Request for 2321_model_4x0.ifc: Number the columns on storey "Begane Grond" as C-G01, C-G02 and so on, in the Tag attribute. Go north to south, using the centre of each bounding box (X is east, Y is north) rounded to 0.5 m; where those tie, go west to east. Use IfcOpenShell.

First a look at what the model holds.

```python
import ifcopenshell
import ifcopenshell.util.element
import ifcopenshell.util.placement

model = ifcopenshell.open("2321_model_4x0.ifc")
print(model.schema)
storey = next(s for s in model.by_type("IfcBuildingStorey") if s.Name == "Begane Grond")
columns = [e for e in ifcopenshell.util.element.get_decomposition(storey) if e.is_a("IfcColumn")]
for e in sorted(columns, key=lambda e: e.id()):
    origin = ifcopenshell.util.placement.get_local_placement(e.ObjectPlacement)[:3, 3]
    print(e.id(), e.Tag, e.Name, origin.round(2) + 0.0, sep=" | ")
```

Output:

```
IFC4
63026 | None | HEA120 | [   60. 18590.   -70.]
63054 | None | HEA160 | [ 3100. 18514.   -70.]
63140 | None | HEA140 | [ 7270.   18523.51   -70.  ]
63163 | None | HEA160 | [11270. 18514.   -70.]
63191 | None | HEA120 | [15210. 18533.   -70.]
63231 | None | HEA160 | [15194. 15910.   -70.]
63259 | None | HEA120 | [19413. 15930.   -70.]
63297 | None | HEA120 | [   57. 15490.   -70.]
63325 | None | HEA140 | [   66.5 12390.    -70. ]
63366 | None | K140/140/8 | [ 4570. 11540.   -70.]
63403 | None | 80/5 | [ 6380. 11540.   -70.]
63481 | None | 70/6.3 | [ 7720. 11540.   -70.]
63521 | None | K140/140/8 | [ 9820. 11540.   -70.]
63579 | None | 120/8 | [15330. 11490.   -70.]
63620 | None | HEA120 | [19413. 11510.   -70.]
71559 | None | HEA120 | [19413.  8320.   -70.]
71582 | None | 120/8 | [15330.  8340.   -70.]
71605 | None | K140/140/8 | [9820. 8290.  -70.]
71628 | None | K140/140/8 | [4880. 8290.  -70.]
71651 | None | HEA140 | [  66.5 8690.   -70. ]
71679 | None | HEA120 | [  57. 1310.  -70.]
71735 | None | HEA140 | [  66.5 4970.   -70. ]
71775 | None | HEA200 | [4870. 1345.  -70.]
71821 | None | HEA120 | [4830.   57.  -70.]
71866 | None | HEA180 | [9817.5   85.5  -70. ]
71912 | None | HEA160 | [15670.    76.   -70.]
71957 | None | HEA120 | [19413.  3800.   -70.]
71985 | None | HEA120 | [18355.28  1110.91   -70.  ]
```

```python
import ifcopenshell
import ifcopenshell.geom
import ifcopenshell.util.element
import ifcopenshell.util.shape

model = ifcopenshell.open("2321_model_4x0.ifc")
settings = ifcopenshell.geom.settings()
settings.set("use-world-coords", True)


def centre(element):
    shape = ifcopenshell.geom.create_shape(settings, element)
    return ifcopenshell.util.shape.get_bbox_centroid(shape.geometry)


storey = next(s for s in model.by_type("IfcBuildingStorey") if s.Name == "Begane Grond")
columns = [e for e in ifcopenshell.util.element.get_decomposition(storey) if e.is_a("IfcColumn")]

# Insertion points can sit at a corner or the storey origin, so sort by the geometry (in metres).
centres = {e: centre(e) for e in columns}
columns.sort(key=lambda e: (-round(centres[e][1] / 0.5), centres[e][0]))

for i, e in enumerate(columns, start=1):
    number = f"C-G{i:02d}"
    e.Tag = number
    print(e.id(), number)

model.write("2321_model_4x0_v2.ifc")
```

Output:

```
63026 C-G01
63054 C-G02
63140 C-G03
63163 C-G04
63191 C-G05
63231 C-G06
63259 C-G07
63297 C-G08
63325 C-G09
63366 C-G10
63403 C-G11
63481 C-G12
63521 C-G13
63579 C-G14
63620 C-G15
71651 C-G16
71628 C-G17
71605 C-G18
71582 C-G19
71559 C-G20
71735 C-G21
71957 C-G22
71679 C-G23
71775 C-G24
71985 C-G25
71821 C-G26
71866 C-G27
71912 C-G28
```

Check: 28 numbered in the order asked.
